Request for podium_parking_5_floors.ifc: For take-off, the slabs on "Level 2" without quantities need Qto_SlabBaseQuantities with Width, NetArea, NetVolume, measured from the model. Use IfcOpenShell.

First a look at what the model holds.

```python
import ifcopenshell
import ifcopenshell.util.element
import ifcopenshell.util.unit

model = ifcopenshell.open("podium_parking_5_floors.ifc")
print(model.schema)
for unit_type in ("LENGTHUNIT", "AREAUNIT", "VOLUMEUNIT"):
    print(unit_type, ifcopenshell.util.unit.calculate_unit_scale(model, unit_type))
storey = next(s for s in model.by_type("IfcBuildingStorey") if s.Name == "Level 2")
slabs = [e for e in ifcopenshell.util.element.get_decomposition(storey) if e.is_a("IfcSlab")]
for e in sorted(slabs, key=lambda e: e.id()):
    print(e.id(), e.is_a(), e.Name, list(ifcopenshell.util.element.get_psets(e, qtos_only=True)), sep=" | ")
```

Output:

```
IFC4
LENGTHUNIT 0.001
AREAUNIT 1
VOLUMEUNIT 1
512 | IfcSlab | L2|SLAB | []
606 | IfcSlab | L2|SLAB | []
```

```python
import ifcopenshell
import ifcopenshell.api.pset
import ifcopenshell.geom
import ifcopenshell.util.element
import ifcopenshell.util.shape
import ifcopenshell.util.unit

model = ifcopenshell.open("podium_parking_5_floors.ifc")
unit_scale = ifcopenshell.util.unit.calculate_unit_scale(model)
area_scale = ifcopenshell.util.unit.calculate_unit_scale(model, "AREAUNIT")
volume_scale = ifcopenshell.util.unit.calculate_unit_scale(model, "VOLUMEUNIT")
settings = ifcopenshell.geom.settings()

storey = next(s for s in model.by_type("IfcBuildingStorey") if s.Name == "Level 2")
slabs = [e for e in ifcopenshell.util.element.get_decomposition(storey) if e.is_a("IfcSlab")]

for e in sorted(slabs, key=lambda e: e.id()):
    if ifcopenshell.util.element.get_psets(e, qtos_only=True, should_inherit=False):
        continue
    # Geometry comes back in metres, in the element's own axes.
    shape = ifcopenshell.geom.create_shape(settings, e)
    values = {
        "Width": ifcopenshell.util.shape.get_z(shape.geometry) / unit_scale,
        "NetArea": ifcopenshell.util.shape.get_footprint_area(shape.geometry) / area_scale,
        "NetVolume": ifcopenshell.util.shape.get_volume(shape.geometry) / volume_scale,
    }
    qto = ifcopenshell.api.pset.add_qto(model, product=e, name="Qto_SlabBaseQuantities")
    ifcopenshell.api.pset.edit_qto(model, qto=qto, properties=values)
    print(e.id(), {k: round(v, 3) for k, v in values.items()})

model.write("podium_parking_5_floors_updated.ifc")
```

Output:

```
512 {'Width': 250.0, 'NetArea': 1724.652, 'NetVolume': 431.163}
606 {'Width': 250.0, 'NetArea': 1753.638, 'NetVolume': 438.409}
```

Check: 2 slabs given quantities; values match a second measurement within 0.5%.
